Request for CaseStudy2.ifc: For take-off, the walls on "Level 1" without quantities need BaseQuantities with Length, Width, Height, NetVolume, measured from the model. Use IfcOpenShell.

First a look at what the model holds.

```python
import ifcopenshell
import ifcopenshell.util.element
import ifcopenshell.util.unit

model = ifcopenshell.open("CaseStudy2.ifc")
print(model.schema)
for unit_type in ("LENGTHUNIT", "AREAUNIT", "VOLUMEUNIT"):
    print(unit_type, ifcopenshell.util.unit.calculate_unit_scale(model, unit_type))
storey = next(s for s in model.by_type("IfcBuildingStorey") if s.Name == "Level 1")
walls = [e for e in ifcopenshell.util.element.get_decomposition(storey) if e.is_a("IfcWall")]
for e in sorted(walls, key=lambda e: e.id()):
    print(e.id(), e.is_a(), e.Name, list(ifcopenshell.util.element.get_psets(e, qtos_only=True)), sep=" | ")
```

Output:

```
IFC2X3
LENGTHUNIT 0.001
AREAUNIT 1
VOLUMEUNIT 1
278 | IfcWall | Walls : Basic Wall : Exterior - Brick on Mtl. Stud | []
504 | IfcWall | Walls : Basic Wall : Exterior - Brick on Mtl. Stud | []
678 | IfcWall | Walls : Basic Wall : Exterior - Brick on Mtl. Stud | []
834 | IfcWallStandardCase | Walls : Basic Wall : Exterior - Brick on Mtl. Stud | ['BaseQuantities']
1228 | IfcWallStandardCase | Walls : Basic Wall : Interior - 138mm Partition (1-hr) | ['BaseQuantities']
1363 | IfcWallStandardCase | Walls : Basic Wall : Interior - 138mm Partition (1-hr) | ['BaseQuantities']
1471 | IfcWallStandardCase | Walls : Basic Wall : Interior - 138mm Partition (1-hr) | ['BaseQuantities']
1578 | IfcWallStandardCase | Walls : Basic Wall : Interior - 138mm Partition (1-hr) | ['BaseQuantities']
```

```python
import ifcopenshell
import ifcopenshell.api.pset
import ifcopenshell.geom
import ifcopenshell.util.element
import ifcopenshell.util.shape
import ifcopenshell.util.unit

model = ifcopenshell.open("CaseStudy2.ifc")
unit_scale = ifcopenshell.util.unit.calculate_unit_scale(model)
volume_scale = ifcopenshell.util.unit.calculate_unit_scale(model, "VOLUMEUNIT")
settings = ifcopenshell.geom.settings()

storey = next(s for s in model.by_type("IfcBuildingStorey") if s.Name == "Level 1")
walls = [e for e in ifcopenshell.util.element.get_decomposition(storey) if e.is_a("IfcWall")]

for e in sorted(walls, key=lambda e: e.id()):
    if ifcopenshell.util.element.get_psets(e, qtos_only=True, should_inherit=False):
        continue
    # Geometry comes back in metres, in the element's own axes.
    shape = ifcopenshell.geom.create_shape(settings, e)
    values = {
        "Length": ifcopenshell.util.shape.get_x(shape.geometry) / unit_scale,
        "Width": ifcopenshell.util.shape.get_y(shape.geometry) / unit_scale,
        "Height": ifcopenshell.util.shape.get_z(shape.geometry) / unit_scale,
        "NetVolume": ifcopenshell.util.shape.get_volume(shape.geometry) / volume_scale,
    }
    qto = ifcopenshell.api.pset.add_qto(model, product=e, name="BaseQuantities")
    ifcopenshell.api.pset.edit_qto(model, qto=qto, properties=values)
    print(e.id(), {k: round(v, 3) for k, v in values.items()})

model.write("CaseStudy2_v2.ifc")
```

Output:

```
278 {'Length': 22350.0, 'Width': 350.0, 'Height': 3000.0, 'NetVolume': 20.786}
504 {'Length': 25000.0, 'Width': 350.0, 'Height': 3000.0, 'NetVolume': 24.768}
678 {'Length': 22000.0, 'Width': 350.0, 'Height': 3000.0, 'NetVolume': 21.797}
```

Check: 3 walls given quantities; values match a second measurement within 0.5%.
